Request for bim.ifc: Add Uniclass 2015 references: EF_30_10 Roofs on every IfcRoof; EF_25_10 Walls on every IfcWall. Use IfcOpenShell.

First a look at what the model holds.

```python
import ifcopenshell

model = ifcopenshell.open("bim.ifc")
print(model.schema)
print("classifications:", [c.Name for c in model.by_type("IfcClassification")])
for ifc_class in ("IfcDoor", "IfcRoof", "IfcStair", "IfcWall", "IfcWindow"):
    print(ifc_class, len(model.by_type(ifc_class)))
```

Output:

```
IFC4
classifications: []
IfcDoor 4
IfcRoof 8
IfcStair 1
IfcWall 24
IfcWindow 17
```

```python
import ifcopenshell
import ifcopenshell.api.classification

model = ifcopenshell.open("bim.ifc")

system = ifcopenshell.api.classification.add_classification(model, classification="Uniclass 2015")

codes = {
    "IfcRoof": ("EF_30_10", "Roofs"),
    "IfcWall": ("EF_25_10", "Walls"),
}
for ifc_class, (code, name) in codes.items():
    products = model.by_type(ifc_class)
    ifcopenshell.api.classification.add_reference(
        model, products=products, classification=system, identification=code, name=name
    )
    print(code, len(products))

model.write("bim_edited.ifc")
```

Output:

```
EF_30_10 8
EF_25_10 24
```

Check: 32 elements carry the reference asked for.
